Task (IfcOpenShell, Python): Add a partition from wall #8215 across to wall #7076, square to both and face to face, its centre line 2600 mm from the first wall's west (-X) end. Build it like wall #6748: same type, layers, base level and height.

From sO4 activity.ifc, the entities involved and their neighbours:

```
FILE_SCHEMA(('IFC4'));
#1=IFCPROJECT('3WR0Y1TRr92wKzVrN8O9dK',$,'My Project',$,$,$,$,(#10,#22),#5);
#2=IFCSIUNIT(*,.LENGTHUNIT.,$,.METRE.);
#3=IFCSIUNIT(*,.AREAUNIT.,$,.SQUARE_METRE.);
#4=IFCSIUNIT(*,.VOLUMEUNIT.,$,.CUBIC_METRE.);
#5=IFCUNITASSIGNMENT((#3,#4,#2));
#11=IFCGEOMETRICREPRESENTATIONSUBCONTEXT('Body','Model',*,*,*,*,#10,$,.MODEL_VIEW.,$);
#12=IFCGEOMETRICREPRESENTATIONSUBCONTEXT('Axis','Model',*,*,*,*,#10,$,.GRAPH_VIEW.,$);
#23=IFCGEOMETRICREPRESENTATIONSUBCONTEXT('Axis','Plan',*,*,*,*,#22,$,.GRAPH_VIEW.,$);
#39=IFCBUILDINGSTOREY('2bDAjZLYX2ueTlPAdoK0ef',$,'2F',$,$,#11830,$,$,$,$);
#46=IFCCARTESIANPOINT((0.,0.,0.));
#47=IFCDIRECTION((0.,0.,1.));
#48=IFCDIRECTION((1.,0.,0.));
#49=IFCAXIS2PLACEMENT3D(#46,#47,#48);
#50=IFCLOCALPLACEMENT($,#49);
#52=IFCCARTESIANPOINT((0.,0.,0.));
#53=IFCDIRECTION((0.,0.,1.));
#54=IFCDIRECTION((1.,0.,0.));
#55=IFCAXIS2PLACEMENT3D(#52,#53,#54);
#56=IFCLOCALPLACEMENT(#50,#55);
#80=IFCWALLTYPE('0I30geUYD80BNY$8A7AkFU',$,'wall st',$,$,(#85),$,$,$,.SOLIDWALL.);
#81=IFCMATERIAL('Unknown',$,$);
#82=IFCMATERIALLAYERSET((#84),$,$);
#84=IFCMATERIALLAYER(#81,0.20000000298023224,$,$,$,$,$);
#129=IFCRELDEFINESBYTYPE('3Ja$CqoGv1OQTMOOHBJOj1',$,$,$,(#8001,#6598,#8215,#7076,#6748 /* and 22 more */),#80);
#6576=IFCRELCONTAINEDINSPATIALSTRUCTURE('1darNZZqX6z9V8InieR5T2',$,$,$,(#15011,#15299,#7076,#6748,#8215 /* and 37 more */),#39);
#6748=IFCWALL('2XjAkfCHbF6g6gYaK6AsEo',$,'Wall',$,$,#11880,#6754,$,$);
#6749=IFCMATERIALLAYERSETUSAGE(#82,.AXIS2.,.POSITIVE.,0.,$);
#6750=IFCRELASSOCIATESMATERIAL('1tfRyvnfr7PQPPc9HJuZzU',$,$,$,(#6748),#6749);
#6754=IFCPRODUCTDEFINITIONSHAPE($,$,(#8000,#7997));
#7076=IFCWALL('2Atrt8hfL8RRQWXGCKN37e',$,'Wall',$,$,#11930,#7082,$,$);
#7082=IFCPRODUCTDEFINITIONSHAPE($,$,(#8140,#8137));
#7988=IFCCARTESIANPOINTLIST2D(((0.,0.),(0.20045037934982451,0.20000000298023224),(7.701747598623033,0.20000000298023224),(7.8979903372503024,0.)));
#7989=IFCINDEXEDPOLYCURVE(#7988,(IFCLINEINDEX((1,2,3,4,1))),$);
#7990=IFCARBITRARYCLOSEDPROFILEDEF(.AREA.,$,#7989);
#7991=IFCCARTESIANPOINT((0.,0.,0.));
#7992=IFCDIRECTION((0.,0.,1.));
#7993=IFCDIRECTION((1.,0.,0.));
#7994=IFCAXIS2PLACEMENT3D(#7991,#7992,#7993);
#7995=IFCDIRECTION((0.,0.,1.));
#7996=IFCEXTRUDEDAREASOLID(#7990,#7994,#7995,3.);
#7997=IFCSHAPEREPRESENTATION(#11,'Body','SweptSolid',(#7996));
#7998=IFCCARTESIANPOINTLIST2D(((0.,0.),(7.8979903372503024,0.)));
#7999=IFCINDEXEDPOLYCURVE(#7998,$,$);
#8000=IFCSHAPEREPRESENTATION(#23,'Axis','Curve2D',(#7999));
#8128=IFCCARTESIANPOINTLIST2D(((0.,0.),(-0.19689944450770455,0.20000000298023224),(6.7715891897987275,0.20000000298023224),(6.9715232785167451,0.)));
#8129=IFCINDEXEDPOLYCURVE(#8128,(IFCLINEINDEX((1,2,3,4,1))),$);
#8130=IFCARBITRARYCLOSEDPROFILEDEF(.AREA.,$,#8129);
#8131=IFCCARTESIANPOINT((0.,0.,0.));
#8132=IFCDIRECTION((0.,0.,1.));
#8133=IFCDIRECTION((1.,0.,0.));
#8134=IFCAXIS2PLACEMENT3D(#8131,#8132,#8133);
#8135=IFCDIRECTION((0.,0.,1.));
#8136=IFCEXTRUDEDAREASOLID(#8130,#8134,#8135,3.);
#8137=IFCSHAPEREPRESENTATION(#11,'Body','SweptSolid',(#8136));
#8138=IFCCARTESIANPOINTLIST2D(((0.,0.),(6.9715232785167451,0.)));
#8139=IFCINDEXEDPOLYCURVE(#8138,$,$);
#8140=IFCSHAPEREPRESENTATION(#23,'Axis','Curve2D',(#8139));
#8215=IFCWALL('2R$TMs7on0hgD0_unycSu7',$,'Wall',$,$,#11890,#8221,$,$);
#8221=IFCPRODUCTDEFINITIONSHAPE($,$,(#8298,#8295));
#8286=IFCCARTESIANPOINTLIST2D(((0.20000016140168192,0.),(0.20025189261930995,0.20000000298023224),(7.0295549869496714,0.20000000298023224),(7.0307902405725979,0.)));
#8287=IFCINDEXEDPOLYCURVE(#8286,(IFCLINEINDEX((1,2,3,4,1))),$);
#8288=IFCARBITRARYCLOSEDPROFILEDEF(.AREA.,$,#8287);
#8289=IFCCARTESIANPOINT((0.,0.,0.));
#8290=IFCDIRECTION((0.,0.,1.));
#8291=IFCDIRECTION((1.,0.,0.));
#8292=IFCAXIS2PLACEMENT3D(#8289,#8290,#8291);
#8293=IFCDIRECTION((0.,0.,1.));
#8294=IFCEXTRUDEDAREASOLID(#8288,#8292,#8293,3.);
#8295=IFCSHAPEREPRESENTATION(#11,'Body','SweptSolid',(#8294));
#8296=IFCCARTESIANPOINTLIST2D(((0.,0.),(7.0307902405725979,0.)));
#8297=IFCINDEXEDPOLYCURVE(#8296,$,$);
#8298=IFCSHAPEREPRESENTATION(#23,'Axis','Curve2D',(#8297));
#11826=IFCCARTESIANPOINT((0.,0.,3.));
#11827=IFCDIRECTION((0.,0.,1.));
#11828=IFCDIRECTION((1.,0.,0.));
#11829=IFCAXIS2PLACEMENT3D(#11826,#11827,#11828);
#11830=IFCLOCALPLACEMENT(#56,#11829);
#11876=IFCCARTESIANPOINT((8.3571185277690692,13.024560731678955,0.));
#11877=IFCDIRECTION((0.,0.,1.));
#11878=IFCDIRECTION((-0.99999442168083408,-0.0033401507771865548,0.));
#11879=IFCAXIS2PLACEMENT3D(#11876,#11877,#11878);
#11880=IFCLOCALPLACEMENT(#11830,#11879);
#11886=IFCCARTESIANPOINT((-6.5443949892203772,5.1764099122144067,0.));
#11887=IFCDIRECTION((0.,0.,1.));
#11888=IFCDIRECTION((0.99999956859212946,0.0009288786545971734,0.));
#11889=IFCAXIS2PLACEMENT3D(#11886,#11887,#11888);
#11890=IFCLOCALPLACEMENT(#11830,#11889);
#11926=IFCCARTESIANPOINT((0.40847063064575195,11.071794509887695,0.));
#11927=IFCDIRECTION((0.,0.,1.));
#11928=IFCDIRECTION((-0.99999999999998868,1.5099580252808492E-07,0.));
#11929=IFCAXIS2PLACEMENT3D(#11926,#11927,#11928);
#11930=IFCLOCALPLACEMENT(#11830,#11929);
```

```python
import numpy as np
import ifcopenshell
import ifcopenshell.api.geometry
import ifcopenshell.api.material
import ifcopenshell.api.pset
import ifcopenshell.api.root
import ifcopenshell.api.spatial
import ifcopenshell.api.type
import ifcopenshell.geom
import ifcopenshell.util.element
import ifcopenshell.util.placement
import ifcopenshell.util.representation
import ifcopenshell.util.shape
import ifcopenshell.util.unit

model = ifcopenshell.open("sO4 activity.ifc")
unit_scale = ifcopenshell.util.unit.calculate_unit_scale(model)
settings = ifcopenshell.geom.settings()
settings.set("use-world-coords", True)

start_wall = model.by_guid("2R$TMs7on0hgD0_unycSu7")
end_wall = model.by_guid("2Atrt8hfL8RRQWXGCKN37e")
like = model.by_guid("2XjAkfCHbF6g6gYaK6AsEo")
matrix = ifcopenshell.util.placement.get_local_placement(start_wall.ObjectPlacement)
matrix[:3, 3] *= unit_scale


def extent(element):
    """Bounding box in the first wall's axes, in metres."""
    shape = ifcopenshell.geom.create_shape(settings, element)
    points = (ifcopenshell.util.shape.get_vertices(shape.geometry) - matrix[:3, 3]) @ matrix[:3, :3]
    return points.min(axis=0), points.max(axis=0)


y_start = extent(start_wall)[1][1]
y_end = extent(end_wall)[0][1]
like_min, like_max = extent(like)
length, height = float(abs(y_end - y_start)), float(like_max[2] - like_min[2])
layer_set = ifcopenshell.util.element.get_material(like, should_skip_usage=True)
thickness = sum(layer.LayerThickness for layer in layer_set.MaterialLayers) * unit_scale

wall = ifcopenshell.api.root.create_entity(model, ifc_class="IfcWall", name="New partition")
storey = ifcopenshell.util.element.get_container(like)
ifcopenshell.api.spatial.assign_container(model, products=[wall], relating_structure=storey)
ifcopenshell.api.type.assign_type(
    model, related_objects=[wall], relating_type=ifcopenshell.util.element.get_type(like), should_map_representations=False
)
rel = ifcopenshell.api.material.assign_material(
    model, products=[wall], type="IfcMaterialLayerSetUsage", material=layer_set
)
rel.RelatingMaterial.OffsetFromReferenceLine = -thickness / 2 / unit_scale
pset = ifcopenshell.api.pset.add_pset(model, product=wall, name="Pset_WallCommon")
ifcopenshell.api.pset.edit_pset(model, pset=pset, properties={"IsExternal": False, "LoadBearing": False})

# The axis runs down the middle of the wall.
axis = ifcopenshell.api.geometry.add_axis_representation(
    model, context=ifcopenshell.util.representation.get_context(model, "Model", "Axis"), axis=[(0.0, 0.0), (length, 0.0)]
)
body = ifcopenshell.api.geometry.add_wall_representation(
    model,
    context=ifcopenshell.util.representation.get_context(model, "Model", "Body", "MODEL_VIEW"),
    length=length,
    height=height,
    thickness=thickness,
    offset=-thickness / 2,
)
for representation in (axis, body):
    ifcopenshell.api.geometry.assign_representation(model, product=wall, representation=representation)

placement = matrix @ ifcopenshell.util.placement.rotation(90, "Z")
placement[:, 3] = matrix @ np.array([extent(start_wall)[0][0] + 2.6, y_start, like_min[2], 1.0])
ifcopenshell.api.geometry.edit_object_placement(model, product=wall, matrix=placement)

print(f"partition {length:.3f} m long, {height:.3f} m high, {thickness:.3f} m thick")

model.write("sO4 activity_v2.ifc")
```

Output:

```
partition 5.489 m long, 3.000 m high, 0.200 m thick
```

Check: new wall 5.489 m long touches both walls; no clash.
